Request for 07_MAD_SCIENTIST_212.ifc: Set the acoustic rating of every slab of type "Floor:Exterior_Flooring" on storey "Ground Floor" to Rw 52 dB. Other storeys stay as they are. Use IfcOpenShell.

First a look at what the model holds.

```python
import ifcopenshell
import ifcopenshell.util.element

model = ifcopenshell.open("07_MAD_SCIENTIST_212.ifc")
print(model.schema)
storey = next(s for s in model.by_type("IfcBuildingStorey") if s.Name == "Ground Floor")
slabs = [e for e in ifcopenshell.util.element.get_decomposition(storey) if e.is_a("IfcSlab")]
seen = {}
for e in slabs:
    element_type = ifcopenshell.util.element.get_type(e)
    key = (element_type.Name if element_type != e and element_type else None, ifcopenshell.util.element.get_pset(e, "Pset_SlabCommon", "AcousticRating"))
    seen[key] = seen.get(key, 0) + 1
for (name, value), count in sorted(seen.items(), key=str):
    print(count, "x", name, "|", value)
```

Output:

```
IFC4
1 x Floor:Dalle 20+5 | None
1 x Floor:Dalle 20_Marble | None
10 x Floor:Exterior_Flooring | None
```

```python
import ifcopenshell
import ifcopenshell.api.pset
import ifcopenshell.util.element

model = ifcopenshell.open("07_MAD_SCIENTIST_212.ifc")

storey = next(s for s in model.by_type("IfcBuildingStorey") if s.Name == "Ground Floor")
slabs = [e for e in ifcopenshell.util.element.get_decomposition(storey) if e.is_a("IfcSlab")]

count = 0
for e in slabs:
    element_type = ifcopenshell.util.element.get_type(e)
    if element_type in (None, e) or element_type.Name != "Floor:Exterior_Flooring":
        continue
    # add_pset returns the element's existing set when there is one.
    pset = ifcopenshell.api.pset.add_pset(model, product=e, name="Pset_SlabCommon")
    ifcopenshell.api.pset.edit_pset(model, pset=pset, properties={"AcousticRating": "Rw 52 dB"})
    count += 1

print(count, "slabs updated")

model.write("07_MAD_SCIENTIST_212_updated.ifc")
```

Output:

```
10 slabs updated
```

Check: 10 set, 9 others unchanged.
